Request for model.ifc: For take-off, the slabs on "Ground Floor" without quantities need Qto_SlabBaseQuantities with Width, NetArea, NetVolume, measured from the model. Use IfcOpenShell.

First a look at what the model holds.

```python
import ifcopenshell
import ifcopenshell.util.element
import ifcopenshell.util.unit

model = ifcopenshell.open("model.ifc")
print(model.schema)
for unit_type in ("LENGTHUNIT", "AREAUNIT", "VOLUMEUNIT"):
    print(unit_type, ifcopenshell.util.unit.calculate_unit_scale(model, unit_type))
storey = next(s for s in model.by_type("IfcBuildingStorey") if s.Name == "Ground Floor")
slabs = [e for e in ifcopenshell.util.element.get_decomposition(storey) if e.is_a("IfcSlab")]
for e in sorted(slabs, key=lambda e: e.id()):
    print(e.id(), e.is_a(), e.Name, list(ifcopenshell.util.element.get_psets(e, qtos_only=True)), sep=" | ")
```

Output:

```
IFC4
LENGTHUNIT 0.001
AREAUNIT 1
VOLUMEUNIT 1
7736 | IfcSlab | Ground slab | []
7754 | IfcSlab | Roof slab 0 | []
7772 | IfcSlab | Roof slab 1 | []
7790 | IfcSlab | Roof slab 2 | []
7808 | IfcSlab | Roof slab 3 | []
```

```python
import ifcopenshell
import ifcopenshell.api.pset
import ifcopenshell.geom
import ifcopenshell.util.element
import ifcopenshell.util.shape
import ifcopenshell.util.unit

model = ifcopenshell.open("model.ifc")
unit_scale = ifcopenshell.util.unit.calculate_unit_scale(model)
area_scale = ifcopenshell.util.unit.calculate_unit_scale(model, "AREAUNIT")
volume_scale = ifcopenshell.util.unit.calculate_unit_scale(model, "VOLUMEUNIT")
settings = ifcopenshell.geom.settings()

storey = next(s for s in model.by_type("IfcBuildingStorey") if s.Name == "Ground Floor")
slabs = [e for e in ifcopenshell.util.element.get_decomposition(storey) if e.is_a("IfcSlab")]

for e in sorted(slabs, key=lambda e: e.id()):
    if ifcopenshell.util.element.get_psets(e, qtos_only=True, should_inherit=False):
        continue
    # Geometry comes back in metres, in the element's own axes.
    shape = ifcopenshell.geom.create_shape(settings, e)
    values = {
        "Width": ifcopenshell.util.shape.get_z(shape.geometry) / unit_scale,
        "NetArea": ifcopenshell.util.shape.get_footprint_area(shape.geometry) / area_scale,
        "NetVolume": ifcopenshell.util.shape.get_volume(shape.geometry) / volume_scale,
    }
    qto = ifcopenshell.api.pset.add_qto(model, product=e, name="Qto_SlabBaseQuantities")
    ifcopenshell.api.pset.edit_qto(model, qto=qto, properties=values)
    print(e.id(), {k: round(v, 3) for k, v in values.items()})

model.write("model_rev.ifc")
```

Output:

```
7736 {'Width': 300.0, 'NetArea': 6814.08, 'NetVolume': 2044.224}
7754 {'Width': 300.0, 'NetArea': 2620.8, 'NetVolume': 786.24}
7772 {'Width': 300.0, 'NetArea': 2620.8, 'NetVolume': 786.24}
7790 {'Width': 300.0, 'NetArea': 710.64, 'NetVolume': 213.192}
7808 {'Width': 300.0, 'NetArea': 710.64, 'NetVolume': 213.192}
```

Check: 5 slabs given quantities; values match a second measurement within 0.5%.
